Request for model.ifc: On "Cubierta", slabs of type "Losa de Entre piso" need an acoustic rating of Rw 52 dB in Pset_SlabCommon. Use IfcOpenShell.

First a look at what the model holds.

```python
import ifcopenshell
import ifcopenshell.util.element

model = ifcopenshell.open("model.ifc")
print(model.schema)
storey = next(s for s in model.by_type("IfcBuildingStorey") if s.Name == "Cubierta")
slabs = [e for e in ifcopenshell.util.element.get_decomposition(storey) if e.is_a("IfcSlab")]
seen = {}
for e in slabs:
    element_type = ifcopenshell.util.element.get_type(e)
    key = (element_type.Name if element_type != e and element_type else None, ifcopenshell.util.element.get_pset(e, "Pset_SlabCommon", "AcousticRating"))
    seen[key] = seen.get(key, 0) + 1
for (name, value), count in sorted(seen.items(), key=str):
    print(count, "x", name, "|", value)
```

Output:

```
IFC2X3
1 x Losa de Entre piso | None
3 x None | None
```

```python
import ifcopenshell
import ifcopenshell.api.pset
import ifcopenshell.util.element

model = ifcopenshell.open("model.ifc")

storey = next(s for s in model.by_type("IfcBuildingStorey") if s.Name == "Cubierta")
slabs = [e for e in ifcopenshell.util.element.get_decomposition(storey) if e.is_a("IfcSlab")]

count = 0
for e in slabs:
    element_type = ifcopenshell.util.element.get_type(e)
    if element_type in (None, e) or element_type.Name != "Losa de Entre piso":
        continue
    # add_pset returns the element's existing set when there is one.
    pset = ifcopenshell.api.pset.add_pset(model, product=e, name="Pset_SlabCommon")
    ifcopenshell.api.pset.edit_pset(model, pset=pset, properties={"AcousticRating": "Rw 52 dB"})
    count += 1

print(count, "slabs updated")

model.write("model_edited.ifc")
```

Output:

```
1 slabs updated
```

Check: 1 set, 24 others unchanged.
